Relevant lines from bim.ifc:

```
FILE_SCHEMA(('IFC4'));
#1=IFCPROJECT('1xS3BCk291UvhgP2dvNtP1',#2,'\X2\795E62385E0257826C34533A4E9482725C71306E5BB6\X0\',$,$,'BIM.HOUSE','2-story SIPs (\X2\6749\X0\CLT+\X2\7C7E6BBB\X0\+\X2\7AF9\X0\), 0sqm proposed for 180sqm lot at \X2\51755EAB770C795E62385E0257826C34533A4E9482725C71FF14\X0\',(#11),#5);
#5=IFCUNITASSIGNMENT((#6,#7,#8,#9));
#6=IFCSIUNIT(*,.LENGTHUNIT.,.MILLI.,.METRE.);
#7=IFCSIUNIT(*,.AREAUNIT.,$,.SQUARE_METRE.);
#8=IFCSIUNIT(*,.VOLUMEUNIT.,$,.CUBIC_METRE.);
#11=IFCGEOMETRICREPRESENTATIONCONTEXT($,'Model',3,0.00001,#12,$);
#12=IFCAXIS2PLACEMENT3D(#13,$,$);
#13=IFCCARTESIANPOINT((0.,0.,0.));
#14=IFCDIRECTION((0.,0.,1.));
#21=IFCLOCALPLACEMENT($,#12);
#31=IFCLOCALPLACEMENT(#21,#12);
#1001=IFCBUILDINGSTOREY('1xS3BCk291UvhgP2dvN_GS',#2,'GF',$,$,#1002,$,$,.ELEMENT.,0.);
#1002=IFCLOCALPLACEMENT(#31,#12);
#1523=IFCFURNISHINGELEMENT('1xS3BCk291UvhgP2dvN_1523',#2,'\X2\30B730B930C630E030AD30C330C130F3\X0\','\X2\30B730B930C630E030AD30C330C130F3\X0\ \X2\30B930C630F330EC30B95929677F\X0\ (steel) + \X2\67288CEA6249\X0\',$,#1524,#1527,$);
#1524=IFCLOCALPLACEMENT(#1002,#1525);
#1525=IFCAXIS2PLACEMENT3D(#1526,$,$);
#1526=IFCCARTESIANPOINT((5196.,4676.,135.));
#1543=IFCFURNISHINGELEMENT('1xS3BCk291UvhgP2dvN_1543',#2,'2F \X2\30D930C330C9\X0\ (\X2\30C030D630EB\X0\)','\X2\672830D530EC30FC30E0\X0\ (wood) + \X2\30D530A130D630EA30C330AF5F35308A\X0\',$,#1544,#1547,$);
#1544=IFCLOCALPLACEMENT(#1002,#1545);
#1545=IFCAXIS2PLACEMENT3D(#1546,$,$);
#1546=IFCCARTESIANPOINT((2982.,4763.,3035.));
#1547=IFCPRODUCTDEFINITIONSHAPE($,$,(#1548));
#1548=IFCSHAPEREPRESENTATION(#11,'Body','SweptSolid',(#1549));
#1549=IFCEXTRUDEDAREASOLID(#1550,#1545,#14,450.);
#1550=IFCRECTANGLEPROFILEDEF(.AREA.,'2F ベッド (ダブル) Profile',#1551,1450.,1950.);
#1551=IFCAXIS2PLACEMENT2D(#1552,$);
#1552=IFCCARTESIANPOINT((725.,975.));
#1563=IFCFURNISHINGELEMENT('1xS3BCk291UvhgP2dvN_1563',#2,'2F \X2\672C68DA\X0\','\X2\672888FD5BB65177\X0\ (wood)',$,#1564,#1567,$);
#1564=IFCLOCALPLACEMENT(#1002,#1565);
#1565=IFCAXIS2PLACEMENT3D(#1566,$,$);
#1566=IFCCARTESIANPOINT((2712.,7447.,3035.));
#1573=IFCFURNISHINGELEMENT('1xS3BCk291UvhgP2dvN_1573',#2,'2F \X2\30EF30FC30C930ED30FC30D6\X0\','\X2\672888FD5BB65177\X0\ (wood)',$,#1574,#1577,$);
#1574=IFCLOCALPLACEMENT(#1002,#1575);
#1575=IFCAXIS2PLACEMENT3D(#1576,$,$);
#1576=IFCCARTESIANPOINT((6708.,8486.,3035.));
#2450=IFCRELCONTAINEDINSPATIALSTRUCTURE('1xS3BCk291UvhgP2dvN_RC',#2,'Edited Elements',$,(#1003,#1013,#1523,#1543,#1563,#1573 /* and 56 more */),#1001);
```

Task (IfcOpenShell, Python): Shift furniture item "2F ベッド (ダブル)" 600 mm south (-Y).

```python
import ifcopenshell
import ifcopenshell.api.geometry
import ifcopenshell.util.placement
import ifcopenshell.util.unit

model = ifcopenshell.open("bim.ifc")
unit_scale = ifcopenshell.util.unit.calculate_unit_scale(model)

item = model.by_guid("1xS3BCk291UvhgP2dvN_1543")
matrix = ifcopenshell.util.placement.get_local_placement(item.ObjectPlacement)
matrix[1, 3] -= 0.6 / unit_scale
ifcopenshell.api.geometry.edit_object_placement(model, product=item, matrix=matrix, is_si=False)

print(ifcopenshell.util.placement.get_local_placement(item.ObjectPlacement).round(3) + 0.0)

model.write("bim_edited.ifc")
```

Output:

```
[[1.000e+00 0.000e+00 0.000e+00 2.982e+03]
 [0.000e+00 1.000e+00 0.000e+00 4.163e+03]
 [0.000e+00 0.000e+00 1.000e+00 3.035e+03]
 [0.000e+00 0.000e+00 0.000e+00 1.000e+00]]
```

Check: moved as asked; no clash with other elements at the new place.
